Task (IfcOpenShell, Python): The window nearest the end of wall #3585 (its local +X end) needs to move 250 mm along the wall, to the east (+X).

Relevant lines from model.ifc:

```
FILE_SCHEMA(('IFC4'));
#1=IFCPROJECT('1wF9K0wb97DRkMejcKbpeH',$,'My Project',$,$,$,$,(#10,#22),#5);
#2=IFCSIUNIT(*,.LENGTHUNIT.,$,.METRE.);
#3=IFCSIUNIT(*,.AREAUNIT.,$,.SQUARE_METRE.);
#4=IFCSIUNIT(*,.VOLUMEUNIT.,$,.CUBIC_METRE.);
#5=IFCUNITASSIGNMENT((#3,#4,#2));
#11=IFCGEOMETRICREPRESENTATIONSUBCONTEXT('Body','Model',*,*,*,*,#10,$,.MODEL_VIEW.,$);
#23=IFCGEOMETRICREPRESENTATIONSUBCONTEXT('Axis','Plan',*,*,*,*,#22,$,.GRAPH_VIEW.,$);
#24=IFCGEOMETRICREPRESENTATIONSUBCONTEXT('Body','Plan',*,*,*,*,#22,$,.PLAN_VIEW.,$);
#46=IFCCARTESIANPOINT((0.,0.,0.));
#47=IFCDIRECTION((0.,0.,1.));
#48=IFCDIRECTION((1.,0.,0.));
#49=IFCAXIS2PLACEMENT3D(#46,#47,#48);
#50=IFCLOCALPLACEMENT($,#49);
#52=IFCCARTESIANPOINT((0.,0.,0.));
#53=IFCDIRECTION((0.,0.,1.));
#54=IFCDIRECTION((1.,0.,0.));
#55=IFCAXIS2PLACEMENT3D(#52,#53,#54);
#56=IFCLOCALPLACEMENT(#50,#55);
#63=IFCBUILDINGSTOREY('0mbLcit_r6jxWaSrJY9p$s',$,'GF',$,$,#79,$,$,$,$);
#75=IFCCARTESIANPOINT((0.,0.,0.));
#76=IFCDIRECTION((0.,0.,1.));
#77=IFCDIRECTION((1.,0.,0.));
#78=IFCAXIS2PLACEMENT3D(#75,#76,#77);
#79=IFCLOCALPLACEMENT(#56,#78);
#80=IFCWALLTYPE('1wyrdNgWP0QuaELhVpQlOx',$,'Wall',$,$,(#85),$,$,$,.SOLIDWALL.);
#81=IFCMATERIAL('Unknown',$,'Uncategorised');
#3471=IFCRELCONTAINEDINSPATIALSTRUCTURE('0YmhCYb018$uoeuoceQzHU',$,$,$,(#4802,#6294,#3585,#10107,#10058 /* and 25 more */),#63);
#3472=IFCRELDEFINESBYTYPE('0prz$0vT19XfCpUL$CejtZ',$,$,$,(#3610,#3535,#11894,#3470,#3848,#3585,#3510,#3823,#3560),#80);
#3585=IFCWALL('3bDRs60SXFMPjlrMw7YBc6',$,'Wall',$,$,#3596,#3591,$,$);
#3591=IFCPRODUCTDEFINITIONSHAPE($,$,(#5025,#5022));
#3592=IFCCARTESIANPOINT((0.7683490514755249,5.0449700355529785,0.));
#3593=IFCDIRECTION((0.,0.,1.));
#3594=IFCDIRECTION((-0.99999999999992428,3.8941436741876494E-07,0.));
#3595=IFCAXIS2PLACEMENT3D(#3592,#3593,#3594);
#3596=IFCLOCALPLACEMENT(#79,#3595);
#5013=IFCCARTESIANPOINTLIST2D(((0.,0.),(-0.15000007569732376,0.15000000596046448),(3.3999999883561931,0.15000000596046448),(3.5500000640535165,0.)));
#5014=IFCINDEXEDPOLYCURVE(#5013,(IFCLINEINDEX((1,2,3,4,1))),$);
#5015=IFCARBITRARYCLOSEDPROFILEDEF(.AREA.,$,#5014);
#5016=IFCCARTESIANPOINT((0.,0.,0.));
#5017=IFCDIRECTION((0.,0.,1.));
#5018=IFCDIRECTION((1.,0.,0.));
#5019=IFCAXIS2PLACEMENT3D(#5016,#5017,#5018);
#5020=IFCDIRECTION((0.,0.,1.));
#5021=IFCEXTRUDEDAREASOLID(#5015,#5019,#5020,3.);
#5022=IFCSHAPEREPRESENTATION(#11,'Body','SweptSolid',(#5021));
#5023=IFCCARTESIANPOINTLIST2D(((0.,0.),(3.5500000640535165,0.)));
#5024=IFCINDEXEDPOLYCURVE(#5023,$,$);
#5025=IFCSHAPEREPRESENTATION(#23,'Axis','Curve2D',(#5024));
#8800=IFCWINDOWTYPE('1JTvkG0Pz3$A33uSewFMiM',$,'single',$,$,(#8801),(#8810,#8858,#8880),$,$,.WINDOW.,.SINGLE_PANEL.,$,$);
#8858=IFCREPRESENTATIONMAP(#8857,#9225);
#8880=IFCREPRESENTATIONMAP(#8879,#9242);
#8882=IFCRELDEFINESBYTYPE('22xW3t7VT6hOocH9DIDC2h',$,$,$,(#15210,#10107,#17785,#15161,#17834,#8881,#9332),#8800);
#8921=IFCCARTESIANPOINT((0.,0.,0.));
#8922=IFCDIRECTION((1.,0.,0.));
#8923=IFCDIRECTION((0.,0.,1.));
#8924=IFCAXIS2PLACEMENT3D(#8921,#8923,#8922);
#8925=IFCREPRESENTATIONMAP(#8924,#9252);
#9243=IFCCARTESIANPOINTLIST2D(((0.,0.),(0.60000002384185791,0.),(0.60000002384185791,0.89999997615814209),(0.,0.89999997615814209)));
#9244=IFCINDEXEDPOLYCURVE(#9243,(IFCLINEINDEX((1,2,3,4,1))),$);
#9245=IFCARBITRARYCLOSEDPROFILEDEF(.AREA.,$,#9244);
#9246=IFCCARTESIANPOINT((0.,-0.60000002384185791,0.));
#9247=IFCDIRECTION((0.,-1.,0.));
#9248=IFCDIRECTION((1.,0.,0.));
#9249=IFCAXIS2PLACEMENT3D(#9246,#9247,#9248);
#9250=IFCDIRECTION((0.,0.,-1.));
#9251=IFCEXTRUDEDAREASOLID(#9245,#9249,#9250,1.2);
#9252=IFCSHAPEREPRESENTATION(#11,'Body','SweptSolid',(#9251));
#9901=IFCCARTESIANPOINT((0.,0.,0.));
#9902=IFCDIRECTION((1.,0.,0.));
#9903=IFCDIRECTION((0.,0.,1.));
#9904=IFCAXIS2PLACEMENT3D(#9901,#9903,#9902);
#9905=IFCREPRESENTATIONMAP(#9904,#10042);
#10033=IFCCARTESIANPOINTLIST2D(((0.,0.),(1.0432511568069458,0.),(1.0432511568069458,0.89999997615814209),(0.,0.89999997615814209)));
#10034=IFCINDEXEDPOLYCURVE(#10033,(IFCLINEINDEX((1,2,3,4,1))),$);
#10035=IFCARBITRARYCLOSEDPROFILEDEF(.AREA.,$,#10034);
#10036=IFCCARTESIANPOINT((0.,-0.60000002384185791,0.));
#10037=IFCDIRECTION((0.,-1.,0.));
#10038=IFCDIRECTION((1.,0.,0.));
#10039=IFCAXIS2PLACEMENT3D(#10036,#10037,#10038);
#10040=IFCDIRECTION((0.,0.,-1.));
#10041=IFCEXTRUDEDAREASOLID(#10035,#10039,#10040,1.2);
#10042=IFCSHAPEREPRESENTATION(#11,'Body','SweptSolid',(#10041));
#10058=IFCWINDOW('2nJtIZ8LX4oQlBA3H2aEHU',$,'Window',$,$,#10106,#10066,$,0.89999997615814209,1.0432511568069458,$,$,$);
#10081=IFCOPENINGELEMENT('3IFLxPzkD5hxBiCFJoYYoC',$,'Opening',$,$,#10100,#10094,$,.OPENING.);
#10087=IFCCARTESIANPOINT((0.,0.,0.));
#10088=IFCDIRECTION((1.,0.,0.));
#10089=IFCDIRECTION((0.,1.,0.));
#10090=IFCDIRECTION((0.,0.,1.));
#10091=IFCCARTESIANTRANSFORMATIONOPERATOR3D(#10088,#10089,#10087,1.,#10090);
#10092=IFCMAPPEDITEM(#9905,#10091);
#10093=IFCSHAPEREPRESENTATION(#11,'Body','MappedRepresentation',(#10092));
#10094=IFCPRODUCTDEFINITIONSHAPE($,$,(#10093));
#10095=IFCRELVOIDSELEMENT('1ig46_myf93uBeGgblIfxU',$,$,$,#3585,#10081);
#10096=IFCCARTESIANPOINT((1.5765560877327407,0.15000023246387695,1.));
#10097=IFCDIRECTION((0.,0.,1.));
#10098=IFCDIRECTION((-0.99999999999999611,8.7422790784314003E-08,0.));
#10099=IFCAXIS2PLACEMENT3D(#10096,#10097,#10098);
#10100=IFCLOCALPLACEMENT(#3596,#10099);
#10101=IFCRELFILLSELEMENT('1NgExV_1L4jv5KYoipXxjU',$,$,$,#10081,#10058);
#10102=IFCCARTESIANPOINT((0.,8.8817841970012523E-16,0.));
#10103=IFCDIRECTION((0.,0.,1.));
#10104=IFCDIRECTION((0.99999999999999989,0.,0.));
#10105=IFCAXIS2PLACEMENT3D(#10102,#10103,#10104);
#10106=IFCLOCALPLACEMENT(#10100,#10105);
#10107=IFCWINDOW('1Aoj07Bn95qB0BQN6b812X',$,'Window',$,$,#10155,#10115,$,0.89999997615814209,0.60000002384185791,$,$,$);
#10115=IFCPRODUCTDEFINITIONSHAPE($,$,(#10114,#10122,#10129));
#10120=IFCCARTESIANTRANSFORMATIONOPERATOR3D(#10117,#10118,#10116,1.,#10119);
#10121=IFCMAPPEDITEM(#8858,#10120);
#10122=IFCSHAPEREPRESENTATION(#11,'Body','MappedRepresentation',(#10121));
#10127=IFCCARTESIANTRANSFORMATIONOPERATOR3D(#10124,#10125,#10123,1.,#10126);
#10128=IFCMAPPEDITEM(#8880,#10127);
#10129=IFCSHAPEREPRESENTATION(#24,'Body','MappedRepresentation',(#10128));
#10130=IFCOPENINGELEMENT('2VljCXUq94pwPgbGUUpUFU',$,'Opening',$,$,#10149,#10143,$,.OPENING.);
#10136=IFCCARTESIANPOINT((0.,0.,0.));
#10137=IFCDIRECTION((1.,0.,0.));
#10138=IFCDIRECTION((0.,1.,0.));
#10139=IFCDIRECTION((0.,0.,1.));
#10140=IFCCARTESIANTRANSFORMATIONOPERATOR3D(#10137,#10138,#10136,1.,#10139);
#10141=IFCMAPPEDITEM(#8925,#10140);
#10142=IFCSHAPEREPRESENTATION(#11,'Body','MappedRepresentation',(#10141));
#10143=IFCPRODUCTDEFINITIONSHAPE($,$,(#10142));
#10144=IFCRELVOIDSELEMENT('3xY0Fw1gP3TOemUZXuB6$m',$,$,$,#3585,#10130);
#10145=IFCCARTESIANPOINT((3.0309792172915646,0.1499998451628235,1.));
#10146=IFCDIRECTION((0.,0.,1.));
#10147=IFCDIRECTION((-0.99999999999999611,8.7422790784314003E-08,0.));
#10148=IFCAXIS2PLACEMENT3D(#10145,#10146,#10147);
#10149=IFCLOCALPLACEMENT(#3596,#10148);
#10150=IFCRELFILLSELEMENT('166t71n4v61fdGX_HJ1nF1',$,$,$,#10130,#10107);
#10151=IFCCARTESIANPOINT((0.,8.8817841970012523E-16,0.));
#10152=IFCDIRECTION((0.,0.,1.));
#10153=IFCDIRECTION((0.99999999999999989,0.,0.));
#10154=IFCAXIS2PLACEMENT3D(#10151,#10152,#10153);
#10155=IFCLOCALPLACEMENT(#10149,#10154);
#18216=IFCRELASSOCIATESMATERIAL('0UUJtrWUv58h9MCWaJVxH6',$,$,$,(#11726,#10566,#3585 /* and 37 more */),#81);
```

```python
import ifcopenshell
import ifcopenshell.api.geometry
import ifcopenshell.util.placement
import ifcopenshell.util.unit

model = ifcopenshell.open("model.ifc")
unit_scale = ifcopenshell.util.unit.calculate_unit_scale(model)

window = model.by_guid("1Aoj07Bn95qB0BQN6b812X")
opening = window.FillsVoids[0].RelatingOpeningElement
wall = opening.VoidsElements[0].RelatingBuildingElement

wall_matrix = ifcopenshell.util.placement.get_local_placement(wall.ObjectPlacement)
shift = wall_matrix[:3, 0] * -0.25 / unit_scale
before = ifcopenshell.util.placement.get_local_placement(window.ObjectPlacement)[:3, 3].copy()

# The window is placed relative to its opening, so it follows when the opening moves.
matrix = ifcopenshell.util.placement.get_local_placement(opening.ObjectPlacement)
matrix[:3, 3] += shift
ifcopenshell.api.geometry.edit_object_placement(
    model, product=opening, matrix=matrix, is_si=False, should_transform_children=True
)

after = ifcopenshell.util.placement.get_local_placement(window.ObjectPlacement)[:3, 3]
print("window moved by", (after - before).round(3) + 0.0)

model.write("model-out.ifc")
```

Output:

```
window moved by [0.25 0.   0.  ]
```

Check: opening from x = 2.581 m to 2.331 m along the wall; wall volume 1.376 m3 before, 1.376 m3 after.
